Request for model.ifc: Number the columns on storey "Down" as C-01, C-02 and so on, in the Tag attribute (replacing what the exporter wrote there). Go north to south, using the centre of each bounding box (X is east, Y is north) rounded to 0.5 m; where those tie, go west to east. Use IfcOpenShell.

First a look at what the model holds.

```python
import ifcopenshell
import ifcopenshell.util.element
import ifcopenshell.util.placement

model = ifcopenshell.open("model.ifc")
print(model.schema)
storey = next(s for s in model.by_type("IfcBuildingStorey") if s.Name == "Down")
columns = [e for e in ifcopenshell.util.element.get_decomposition(storey) if e.is_a("IfcColumn")]
for e in sorted(columns, key=lambda e: e.id()):
    origin = ifcopenshell.util.placement.get_local_placement(e.ObjectPlacement)[:3, 3]
    print(e.id(), e.Tag, e.Name, origin.round(2) + 0.0, sep=" | ")
```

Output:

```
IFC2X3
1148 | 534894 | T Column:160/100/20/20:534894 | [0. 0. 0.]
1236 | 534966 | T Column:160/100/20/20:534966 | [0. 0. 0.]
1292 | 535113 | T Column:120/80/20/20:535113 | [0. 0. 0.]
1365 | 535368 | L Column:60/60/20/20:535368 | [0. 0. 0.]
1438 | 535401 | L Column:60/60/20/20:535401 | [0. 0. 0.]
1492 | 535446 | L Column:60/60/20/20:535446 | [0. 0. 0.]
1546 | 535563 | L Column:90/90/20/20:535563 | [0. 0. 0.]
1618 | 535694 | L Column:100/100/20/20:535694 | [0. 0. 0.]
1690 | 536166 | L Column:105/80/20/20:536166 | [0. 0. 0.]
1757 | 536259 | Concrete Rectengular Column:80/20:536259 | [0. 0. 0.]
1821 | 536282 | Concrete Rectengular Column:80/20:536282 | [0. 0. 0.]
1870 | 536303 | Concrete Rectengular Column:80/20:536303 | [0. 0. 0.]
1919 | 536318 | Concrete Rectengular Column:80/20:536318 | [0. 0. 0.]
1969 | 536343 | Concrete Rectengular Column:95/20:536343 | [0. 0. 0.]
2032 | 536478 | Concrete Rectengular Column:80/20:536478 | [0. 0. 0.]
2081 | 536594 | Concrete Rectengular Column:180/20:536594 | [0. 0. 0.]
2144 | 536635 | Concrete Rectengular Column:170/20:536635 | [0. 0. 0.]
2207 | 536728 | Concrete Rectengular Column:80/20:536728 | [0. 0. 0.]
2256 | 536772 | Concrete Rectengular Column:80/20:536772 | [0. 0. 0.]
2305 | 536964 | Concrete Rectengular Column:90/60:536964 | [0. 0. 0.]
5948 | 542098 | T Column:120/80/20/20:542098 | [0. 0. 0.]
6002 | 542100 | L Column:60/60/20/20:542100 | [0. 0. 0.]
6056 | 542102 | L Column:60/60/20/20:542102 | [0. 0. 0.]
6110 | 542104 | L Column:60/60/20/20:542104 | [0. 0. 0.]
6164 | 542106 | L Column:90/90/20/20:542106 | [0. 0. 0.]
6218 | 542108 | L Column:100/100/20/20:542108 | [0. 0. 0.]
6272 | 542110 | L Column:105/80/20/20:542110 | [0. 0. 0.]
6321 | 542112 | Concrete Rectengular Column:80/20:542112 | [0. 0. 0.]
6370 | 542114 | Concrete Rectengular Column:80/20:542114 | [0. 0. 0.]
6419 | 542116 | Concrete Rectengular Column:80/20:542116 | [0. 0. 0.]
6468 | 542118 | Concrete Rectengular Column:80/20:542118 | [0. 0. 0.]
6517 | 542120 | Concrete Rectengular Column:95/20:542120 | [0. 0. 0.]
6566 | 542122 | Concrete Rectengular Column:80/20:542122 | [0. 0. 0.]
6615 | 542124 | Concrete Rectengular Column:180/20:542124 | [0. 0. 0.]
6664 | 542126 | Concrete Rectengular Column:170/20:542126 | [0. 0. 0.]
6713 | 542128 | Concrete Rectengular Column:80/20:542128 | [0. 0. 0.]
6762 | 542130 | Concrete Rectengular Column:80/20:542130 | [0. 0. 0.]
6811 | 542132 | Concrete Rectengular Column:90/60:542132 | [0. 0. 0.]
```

```python
import ifcopenshell
import ifcopenshell.geom
import ifcopenshell.util.element
import ifcopenshell.util.shape

model = ifcopenshell.open("model.ifc")
settings = ifcopenshell.geom.settings()
settings.set("use-world-coords", True)


def centre(element):
    shape = ifcopenshell.geom.create_shape(settings, element)
    return ifcopenshell.util.shape.get_bbox_centroid(shape.geometry)


storey = next(s for s in model.by_type("IfcBuildingStorey") if s.Name == "Down")
columns = [e for e in ifcopenshell.util.element.get_decomposition(storey) if e.is_a("IfcColumn")]

# Insertion points can sit at a corner or the storey origin, so sort by the geometry (in metres).
centres = {e: centre(e) for e in columns}
columns.sort(key=lambda e: (-round(centres[e][1] / 0.5), centres[e][0]))

for i, e in enumerate(columns, start=1):
    number = f"C-{i:02d}"
    e.Tag = number
    print(e.id(), number)

model.write("model_rev.ifc")
```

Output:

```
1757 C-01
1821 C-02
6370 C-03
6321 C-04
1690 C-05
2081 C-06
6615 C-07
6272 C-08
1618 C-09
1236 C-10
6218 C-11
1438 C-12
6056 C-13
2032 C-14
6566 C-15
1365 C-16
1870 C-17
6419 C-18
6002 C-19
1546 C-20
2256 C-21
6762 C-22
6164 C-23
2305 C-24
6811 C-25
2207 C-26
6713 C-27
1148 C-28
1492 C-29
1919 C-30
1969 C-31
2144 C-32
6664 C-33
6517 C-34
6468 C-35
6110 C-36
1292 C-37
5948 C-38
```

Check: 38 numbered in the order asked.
